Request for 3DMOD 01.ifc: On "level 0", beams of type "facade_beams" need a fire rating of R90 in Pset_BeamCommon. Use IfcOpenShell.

First a look at what the model holds.

```python
import ifcopenshell
import ifcopenshell.util.element

model = ifcopenshell.open("3DMOD 01.ifc")
print(model.schema)
storey = next(s for s in model.by_type("IfcBuildingStorey") if s.Name == "level 0")
beams = [e for e in ifcopenshell.util.element.get_decomposition(storey) if e.is_a("IfcBeam")]
seen = {}
for e in beams:
    element_type = ifcopenshell.util.element.get_type(e)
    key = (element_type.Name if element_type != e and element_type else None, ifcopenshell.util.element.get_pset(e, "Pset_BeamCommon", "FireRating"))
    seen[key] = seen.get(key, 0) + 1
for (name, value), count in sorted(seen.items(), key=str):
    print(count, "x", name, "|", value)
```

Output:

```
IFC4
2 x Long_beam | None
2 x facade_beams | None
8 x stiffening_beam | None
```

```python
import ifcopenshell
import ifcopenshell.api.pset
import ifcopenshell.util.element

model = ifcopenshell.open("3DMOD 01.ifc")

storey = next(s for s in model.by_type("IfcBuildingStorey") if s.Name == "level 0")
beams = [e for e in ifcopenshell.util.element.get_decomposition(storey) if e.is_a("IfcBeam")]

count = 0
for e in beams:
    element_type = ifcopenshell.util.element.get_type(e)
    if element_type in (None, e) or element_type.Name != "facade_beams":
        continue
    # add_pset returns the element's existing set when there is one.
    pset = ifcopenshell.api.pset.add_pset(model, product=e, name="Pset_BeamCommon")
    ifcopenshell.api.pset.edit_pset(model, pset=pset, properties={"FireRating": "R90"})
    count += 1

print(count, "beams updated")

model.write("3DMOD 01_v2.ifc")
```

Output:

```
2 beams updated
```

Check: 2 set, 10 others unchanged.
